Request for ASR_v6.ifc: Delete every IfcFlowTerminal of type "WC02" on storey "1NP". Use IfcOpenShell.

First a look at what the model holds.

```python
import ifcopenshell
import ifcopenshell.util.element

model = ifcopenshell.open("ASR_v6.ifc")
print(model.schema)
storey = next(s for s in model.by_type("IfcBuildingStorey") if s.Name == "1NP")
terminals = [e for e in ifcopenshell.util.element.get_decomposition(storey) if e.is_a("IfcFlowTerminal")]
seen = {}
for e in terminals:
    element_type = ifcopenshell.util.element.get_type(e)
    name = element_type.Name if element_type not in (None, e) else None
    seen[name] = seen.get(name, 0) + 1
for name, count in sorted(seen.items(), key=str):
    print(count, "x", name)
```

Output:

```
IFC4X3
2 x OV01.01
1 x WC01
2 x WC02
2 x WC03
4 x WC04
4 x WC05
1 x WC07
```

```python
import ifcopenshell
import ifcopenshell.api.root
import ifcopenshell.util.element

model = ifcopenshell.open("ASR_v6.ifc")

storey = next(s for s in model.by_type("IfcBuildingStorey") if s.Name == "1NP")
terminals = [e for e in ifcopenshell.util.element.get_decomposition(storey) if e.is_a("IfcFlowTerminal")]
targets = [e for e in terminals if (t := ifcopenshell.util.element.get_type(e)) not in (None, e) and t.Name == "WC02"]

for e in targets:
    ifcopenshell.api.root.remove_product(model, product=e)
print(len(targets), "removed")

model.write("ASR_v6_edited.ifc")
```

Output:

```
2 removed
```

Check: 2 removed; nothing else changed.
